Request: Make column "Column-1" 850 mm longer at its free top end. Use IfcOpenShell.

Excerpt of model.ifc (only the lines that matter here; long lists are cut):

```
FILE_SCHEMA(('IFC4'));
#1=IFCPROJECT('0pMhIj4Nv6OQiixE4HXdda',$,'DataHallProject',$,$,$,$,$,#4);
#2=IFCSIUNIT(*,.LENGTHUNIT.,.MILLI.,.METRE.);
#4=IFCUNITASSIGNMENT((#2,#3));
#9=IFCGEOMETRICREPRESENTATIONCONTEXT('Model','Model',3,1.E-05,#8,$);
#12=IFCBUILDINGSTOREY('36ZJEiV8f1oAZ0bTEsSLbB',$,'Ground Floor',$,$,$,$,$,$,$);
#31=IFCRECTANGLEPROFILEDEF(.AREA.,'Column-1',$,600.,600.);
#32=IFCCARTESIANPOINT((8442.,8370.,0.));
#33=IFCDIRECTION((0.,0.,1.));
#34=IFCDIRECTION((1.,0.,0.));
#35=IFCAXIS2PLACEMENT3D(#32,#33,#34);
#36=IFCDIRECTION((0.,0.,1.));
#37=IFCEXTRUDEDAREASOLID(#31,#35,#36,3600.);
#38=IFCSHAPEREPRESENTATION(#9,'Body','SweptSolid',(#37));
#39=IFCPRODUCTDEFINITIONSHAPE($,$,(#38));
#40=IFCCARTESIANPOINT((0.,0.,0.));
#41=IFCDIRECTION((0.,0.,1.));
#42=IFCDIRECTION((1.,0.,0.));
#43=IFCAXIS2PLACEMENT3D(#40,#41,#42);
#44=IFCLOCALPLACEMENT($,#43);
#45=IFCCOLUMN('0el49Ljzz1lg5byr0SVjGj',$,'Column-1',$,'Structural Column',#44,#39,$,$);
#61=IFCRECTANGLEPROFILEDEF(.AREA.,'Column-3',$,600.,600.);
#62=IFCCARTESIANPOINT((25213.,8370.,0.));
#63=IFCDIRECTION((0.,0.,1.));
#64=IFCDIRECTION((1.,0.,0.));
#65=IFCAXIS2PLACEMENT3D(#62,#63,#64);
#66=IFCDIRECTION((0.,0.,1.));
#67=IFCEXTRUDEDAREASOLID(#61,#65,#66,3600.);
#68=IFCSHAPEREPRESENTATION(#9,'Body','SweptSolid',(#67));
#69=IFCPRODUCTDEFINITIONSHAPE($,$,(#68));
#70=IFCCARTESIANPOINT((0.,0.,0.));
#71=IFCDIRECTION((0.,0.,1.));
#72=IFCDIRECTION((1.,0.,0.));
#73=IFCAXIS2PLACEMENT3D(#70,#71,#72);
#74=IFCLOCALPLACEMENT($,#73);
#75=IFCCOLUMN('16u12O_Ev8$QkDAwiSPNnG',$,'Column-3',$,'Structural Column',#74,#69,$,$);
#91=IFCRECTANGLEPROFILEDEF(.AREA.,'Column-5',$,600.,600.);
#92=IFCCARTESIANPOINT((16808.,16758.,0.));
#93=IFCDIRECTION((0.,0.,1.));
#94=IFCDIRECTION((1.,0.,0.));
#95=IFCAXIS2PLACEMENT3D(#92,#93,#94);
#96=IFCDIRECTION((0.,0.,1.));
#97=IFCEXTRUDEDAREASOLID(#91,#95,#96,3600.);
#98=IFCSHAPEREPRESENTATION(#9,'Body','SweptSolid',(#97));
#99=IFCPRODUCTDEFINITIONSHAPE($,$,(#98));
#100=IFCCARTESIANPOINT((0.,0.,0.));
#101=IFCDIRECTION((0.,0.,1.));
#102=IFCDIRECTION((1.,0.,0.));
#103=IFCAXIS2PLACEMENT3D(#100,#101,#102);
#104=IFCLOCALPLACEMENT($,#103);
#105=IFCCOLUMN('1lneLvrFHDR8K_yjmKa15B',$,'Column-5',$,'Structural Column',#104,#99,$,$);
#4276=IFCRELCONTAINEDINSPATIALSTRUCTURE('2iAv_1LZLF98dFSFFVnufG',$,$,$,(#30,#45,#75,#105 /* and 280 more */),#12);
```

```python
import ifcopenshell
import ifcopenshell.util.unit

model = ifcopenshell.open("model.ifc")
unit_scale = ifcopenshell.util.unit.calculate_unit_scale(model)

member = model.by_guid("0el49Ljzz1lg5byr0SVjGj")
change = 0.85 / unit_scale

# The extrusion runs towards the end named, so only its depth changes.
body = next(r for r in member.Representation.Representations if r.RepresentationIdentifier == "Body")
solid = body.Items[0]
old_length = solid.Depth
solid.Depth += change

print(f"length {old_length:g} -> {solid.Depth:g}")

model.write("model_v2.ifc")
```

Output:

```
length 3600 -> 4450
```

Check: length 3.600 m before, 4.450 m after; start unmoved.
